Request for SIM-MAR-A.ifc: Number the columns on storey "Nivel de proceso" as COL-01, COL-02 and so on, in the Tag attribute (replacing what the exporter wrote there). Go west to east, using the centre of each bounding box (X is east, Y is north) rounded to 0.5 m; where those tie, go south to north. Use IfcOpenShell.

First a look at what the model holds.

```python
import ifcopenshell
import ifcopenshell.util.element
import ifcopenshell.util.placement

model = ifcopenshell.open("SIM-MAR-A.ifc")
print(model.schema)
storey = next(s for s in model.by_type("IfcBuildingStorey") if s.Name == "Nivel de proceso")
columns = [e for e in ifcopenshell.util.element.get_decomposition(storey) if e.is_a("IfcColumn")]
for e in sorted(columns, key=lambda e: e.id()):
    origin = ifcopenshell.util.placement.get_local_placement(e.ObjectPlacement)[:3, 3]
    print(e.id(), e.Tag, e.Name, origin.round(2) + 0.0, sep=" | ")
```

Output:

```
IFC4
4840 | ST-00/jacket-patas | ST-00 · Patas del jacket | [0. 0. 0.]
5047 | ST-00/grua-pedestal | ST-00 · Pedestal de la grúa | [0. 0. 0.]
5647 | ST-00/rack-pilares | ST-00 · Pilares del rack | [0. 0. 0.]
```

```python
import ifcopenshell
import ifcopenshell.geom
import ifcopenshell.util.element
import ifcopenshell.util.shape

model = ifcopenshell.open("SIM-MAR-A.ifc")
settings = ifcopenshell.geom.settings()
settings.set("use-world-coords", True)


def centre(element):
    shape = ifcopenshell.geom.create_shape(settings, element)
    return ifcopenshell.util.shape.get_bbox_centroid(shape.geometry)


storey = next(s for s in model.by_type("IfcBuildingStorey") if s.Name == "Nivel de proceso")
columns = [e for e in ifcopenshell.util.element.get_decomposition(storey) if e.is_a("IfcColumn")]

# Insertion points can sit at a corner or the storey origin, so sort by the geometry (in metres).
centres = {e: centre(e) for e in columns}
columns.sort(key=lambda e: (round(centres[e][0] / 0.5), centres[e][1]))

for i, e in enumerate(columns, start=1):
    number = f"COL-{i:02d}"
    e.Tag = number
    print(e.id(), number)

model.write("SIM-MAR-A_updated.ifc")
```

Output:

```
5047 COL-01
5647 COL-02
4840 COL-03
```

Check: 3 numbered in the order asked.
